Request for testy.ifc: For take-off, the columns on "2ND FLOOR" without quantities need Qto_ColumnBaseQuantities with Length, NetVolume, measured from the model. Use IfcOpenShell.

First a look at what the model holds.

```python
import ifcopenshell
import ifcopenshell.util.element
import ifcopenshell.util.unit

model = ifcopenshell.open("testy.ifc")
print(model.schema)
for unit_type in ("LENGTHUNIT", "AREAUNIT", "VOLUMEUNIT"):
    print(unit_type, ifcopenshell.util.unit.calculate_unit_scale(model, unit_type))
storey = next(s for s in model.by_type("IfcBuildingStorey") if s.Name == "2ND FLOOR")
columns = [e for e in ifcopenshell.util.element.get_decomposition(storey) if e.is_a("IfcColumn")]
for e in sorted(columns, key=lambda e: e.id()):
    print(e.id(), e.is_a(), e.Name, list(ifcopenshell.util.element.get_psets(e, qtos_only=True)), sep=" | ")
```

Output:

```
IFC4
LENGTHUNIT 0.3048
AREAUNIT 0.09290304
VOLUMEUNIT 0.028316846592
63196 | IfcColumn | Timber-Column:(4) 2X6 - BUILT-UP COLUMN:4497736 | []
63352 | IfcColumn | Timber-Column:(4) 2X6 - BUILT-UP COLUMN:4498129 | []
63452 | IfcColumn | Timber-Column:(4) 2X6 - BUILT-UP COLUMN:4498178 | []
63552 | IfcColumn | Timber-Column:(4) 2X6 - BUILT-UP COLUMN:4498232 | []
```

```python
import ifcopenshell
import ifcopenshell.api.pset
import ifcopenshell.geom
import ifcopenshell.util.element
import ifcopenshell.util.shape
import ifcopenshell.util.unit

model = ifcopenshell.open("testy.ifc")
unit_scale = ifcopenshell.util.unit.calculate_unit_scale(model)
volume_scale = ifcopenshell.util.unit.calculate_unit_scale(model, "VOLUMEUNIT")
settings = ifcopenshell.geom.settings()

storey = next(s for s in model.by_type("IfcBuildingStorey") if s.Name == "2ND FLOOR")
columns = [e for e in ifcopenshell.util.element.get_decomposition(storey) if e.is_a("IfcColumn")]

for e in sorted(columns, key=lambda e: e.id()):
    if ifcopenshell.util.element.get_psets(e, qtos_only=True, should_inherit=False):
        continue
    # Geometry comes back in metres, in the element's own axes.
    shape = ifcopenshell.geom.create_shape(settings, e)
    values = {
        "Length": ifcopenshell.util.shape.get_z(shape.geometry) / unit_scale,
        "NetVolume": ifcopenshell.util.shape.get_volume(shape.geometry) / volume_scale,
    }
    qto = ifcopenshell.api.pset.add_qto(model, product=e, name="Qto_ColumnBaseQuantities")
    ifcopenshell.api.pset.edit_qto(model, qto=qto, properties=values)
    print(e.id(), {k: round(v, 3) for k, v in values.items()})

model.write("testy_edited.ifc")
```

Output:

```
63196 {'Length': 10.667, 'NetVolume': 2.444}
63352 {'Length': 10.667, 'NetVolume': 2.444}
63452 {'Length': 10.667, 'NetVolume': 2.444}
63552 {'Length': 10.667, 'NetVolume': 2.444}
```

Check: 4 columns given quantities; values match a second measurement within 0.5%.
